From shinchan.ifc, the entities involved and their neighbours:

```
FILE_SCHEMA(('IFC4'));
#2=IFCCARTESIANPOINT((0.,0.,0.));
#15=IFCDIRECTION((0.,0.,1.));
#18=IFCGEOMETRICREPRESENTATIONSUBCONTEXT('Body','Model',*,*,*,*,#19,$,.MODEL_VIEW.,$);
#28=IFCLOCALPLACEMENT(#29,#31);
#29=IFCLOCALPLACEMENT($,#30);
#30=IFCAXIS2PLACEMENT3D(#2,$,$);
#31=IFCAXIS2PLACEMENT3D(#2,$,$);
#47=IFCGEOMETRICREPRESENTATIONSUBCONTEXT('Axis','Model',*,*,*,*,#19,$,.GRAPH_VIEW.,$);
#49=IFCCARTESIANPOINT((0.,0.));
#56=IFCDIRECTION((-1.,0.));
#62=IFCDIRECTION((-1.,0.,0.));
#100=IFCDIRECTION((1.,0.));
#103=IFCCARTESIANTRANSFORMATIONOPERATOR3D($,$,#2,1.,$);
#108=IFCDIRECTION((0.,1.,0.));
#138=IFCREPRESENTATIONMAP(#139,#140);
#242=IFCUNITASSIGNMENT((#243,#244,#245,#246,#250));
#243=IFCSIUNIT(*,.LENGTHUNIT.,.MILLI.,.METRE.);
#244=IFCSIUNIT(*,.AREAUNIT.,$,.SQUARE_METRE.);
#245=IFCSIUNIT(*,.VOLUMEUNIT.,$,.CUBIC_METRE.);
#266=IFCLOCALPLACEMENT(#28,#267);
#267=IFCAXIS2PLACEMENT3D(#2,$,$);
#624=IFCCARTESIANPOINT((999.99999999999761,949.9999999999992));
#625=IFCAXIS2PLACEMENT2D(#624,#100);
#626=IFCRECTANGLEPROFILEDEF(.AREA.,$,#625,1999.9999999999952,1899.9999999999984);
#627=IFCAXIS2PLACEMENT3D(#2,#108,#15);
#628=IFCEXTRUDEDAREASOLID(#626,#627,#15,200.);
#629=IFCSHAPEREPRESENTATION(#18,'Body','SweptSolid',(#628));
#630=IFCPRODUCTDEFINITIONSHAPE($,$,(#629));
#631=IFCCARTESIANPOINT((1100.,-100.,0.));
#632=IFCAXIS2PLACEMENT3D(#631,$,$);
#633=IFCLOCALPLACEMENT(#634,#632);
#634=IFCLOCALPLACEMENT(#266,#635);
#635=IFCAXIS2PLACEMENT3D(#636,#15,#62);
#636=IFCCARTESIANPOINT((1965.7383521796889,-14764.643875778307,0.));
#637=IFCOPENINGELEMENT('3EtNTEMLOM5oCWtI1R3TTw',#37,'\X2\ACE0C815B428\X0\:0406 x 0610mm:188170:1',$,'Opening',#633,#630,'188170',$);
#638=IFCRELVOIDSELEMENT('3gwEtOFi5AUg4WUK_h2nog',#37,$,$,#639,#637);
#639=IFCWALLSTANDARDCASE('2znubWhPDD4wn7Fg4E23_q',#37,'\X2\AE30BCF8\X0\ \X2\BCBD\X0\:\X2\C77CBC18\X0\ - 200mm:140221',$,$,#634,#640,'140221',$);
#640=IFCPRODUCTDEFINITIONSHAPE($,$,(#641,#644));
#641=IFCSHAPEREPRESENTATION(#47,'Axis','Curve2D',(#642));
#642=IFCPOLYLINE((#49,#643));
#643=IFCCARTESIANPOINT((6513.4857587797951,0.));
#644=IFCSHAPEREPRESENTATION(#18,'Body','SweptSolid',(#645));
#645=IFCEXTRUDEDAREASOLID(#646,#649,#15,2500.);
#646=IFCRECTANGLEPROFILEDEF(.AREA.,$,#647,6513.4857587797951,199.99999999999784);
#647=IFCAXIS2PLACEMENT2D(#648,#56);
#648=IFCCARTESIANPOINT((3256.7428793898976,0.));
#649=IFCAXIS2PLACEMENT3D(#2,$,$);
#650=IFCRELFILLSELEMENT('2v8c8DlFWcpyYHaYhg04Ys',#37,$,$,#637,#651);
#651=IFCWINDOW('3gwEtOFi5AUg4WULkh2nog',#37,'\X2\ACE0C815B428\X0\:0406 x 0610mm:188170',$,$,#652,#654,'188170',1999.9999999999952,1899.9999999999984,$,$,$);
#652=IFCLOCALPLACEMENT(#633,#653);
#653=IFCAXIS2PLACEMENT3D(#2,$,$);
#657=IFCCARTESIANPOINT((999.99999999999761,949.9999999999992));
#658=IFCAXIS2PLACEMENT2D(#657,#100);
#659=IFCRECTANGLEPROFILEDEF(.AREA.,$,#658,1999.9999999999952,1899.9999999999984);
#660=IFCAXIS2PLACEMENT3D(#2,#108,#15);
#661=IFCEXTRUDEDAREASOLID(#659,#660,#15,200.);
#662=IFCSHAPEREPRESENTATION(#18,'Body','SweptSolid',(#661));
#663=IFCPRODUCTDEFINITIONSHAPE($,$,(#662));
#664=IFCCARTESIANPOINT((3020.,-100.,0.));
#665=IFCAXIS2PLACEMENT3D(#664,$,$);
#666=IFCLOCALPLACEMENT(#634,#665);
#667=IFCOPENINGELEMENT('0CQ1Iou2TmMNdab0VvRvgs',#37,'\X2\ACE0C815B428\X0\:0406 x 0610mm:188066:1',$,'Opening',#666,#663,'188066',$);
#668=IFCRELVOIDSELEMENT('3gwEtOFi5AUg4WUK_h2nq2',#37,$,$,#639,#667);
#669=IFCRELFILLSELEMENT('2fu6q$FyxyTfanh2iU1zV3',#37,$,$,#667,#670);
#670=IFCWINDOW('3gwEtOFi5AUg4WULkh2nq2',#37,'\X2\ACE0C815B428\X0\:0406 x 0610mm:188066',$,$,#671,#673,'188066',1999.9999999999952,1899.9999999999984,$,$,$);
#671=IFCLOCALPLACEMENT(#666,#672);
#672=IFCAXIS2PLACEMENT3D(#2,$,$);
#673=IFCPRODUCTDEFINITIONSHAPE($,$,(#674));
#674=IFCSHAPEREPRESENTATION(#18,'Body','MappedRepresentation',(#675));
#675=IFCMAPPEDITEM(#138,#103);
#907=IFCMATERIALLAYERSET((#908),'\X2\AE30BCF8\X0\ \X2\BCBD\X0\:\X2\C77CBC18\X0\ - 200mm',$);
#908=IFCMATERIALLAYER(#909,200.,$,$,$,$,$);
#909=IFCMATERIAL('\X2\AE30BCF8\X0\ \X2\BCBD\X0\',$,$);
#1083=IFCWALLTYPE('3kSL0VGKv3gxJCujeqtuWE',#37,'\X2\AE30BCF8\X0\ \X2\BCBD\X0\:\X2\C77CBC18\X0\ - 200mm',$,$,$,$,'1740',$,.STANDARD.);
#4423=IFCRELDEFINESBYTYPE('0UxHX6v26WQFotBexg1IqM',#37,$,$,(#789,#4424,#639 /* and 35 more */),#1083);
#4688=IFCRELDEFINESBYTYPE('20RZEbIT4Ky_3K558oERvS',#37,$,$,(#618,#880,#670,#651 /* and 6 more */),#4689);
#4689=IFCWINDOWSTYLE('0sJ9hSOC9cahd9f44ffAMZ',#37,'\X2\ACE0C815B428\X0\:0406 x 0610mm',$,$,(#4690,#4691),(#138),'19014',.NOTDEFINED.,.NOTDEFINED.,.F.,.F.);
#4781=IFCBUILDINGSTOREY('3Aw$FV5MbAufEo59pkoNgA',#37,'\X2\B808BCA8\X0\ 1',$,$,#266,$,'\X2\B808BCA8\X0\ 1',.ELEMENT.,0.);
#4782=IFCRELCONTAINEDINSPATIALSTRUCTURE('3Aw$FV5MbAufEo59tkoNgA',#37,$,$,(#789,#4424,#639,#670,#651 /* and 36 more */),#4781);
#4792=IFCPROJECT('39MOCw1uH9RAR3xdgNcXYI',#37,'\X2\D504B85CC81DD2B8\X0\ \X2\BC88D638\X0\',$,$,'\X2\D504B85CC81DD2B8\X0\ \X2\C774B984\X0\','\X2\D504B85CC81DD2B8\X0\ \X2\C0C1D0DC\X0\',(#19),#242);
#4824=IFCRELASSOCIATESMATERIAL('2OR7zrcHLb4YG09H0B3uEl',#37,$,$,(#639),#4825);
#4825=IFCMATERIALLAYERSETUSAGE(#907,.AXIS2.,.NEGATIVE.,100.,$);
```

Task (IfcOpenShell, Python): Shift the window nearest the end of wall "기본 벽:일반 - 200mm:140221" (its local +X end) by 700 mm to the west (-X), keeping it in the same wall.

```python
import ifcopenshell
import ifcopenshell.api.geometry
import ifcopenshell.util.placement
import ifcopenshell.util.unit

model = ifcopenshell.open("shinchan.ifc")
unit_scale = ifcopenshell.util.unit.calculate_unit_scale(model)

window = model.by_guid("3gwEtOFi5AUg4WULkh2nq2")
opening = window.FillsVoids[0].RelatingOpeningElement
wall = opening.VoidsElements[0].RelatingBuildingElement

wall_matrix = ifcopenshell.util.placement.get_local_placement(wall.ObjectPlacement)
shift = wall_matrix[:3, 0] * 0.7 / unit_scale
before = ifcopenshell.util.placement.get_local_placement(window.ObjectPlacement)[:3, 3].copy()

# The window is placed relative to its opening, so it follows when the opening moves.
matrix = ifcopenshell.util.placement.get_local_placement(opening.ObjectPlacement)
matrix[:3, 3] += shift
ifcopenshell.api.geometry.edit_object_placement(
    model, product=opening, matrix=matrix, is_si=False, should_transform_children=True
)

after = ifcopenshell.util.placement.get_local_placement(window.ObjectPlacement)[:3, 3]
print("window moved by", (after - before).round(3) + 0.0)

model.write("shinchan_rev.ifc")
```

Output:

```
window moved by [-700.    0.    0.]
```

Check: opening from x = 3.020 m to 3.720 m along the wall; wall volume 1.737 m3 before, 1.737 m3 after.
